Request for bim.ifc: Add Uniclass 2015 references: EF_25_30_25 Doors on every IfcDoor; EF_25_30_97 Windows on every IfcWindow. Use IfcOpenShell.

First a look at what the model holds.

```python
import ifcopenshell

model = ifcopenshell.open("bim.ifc")
print(model.schema)
print("classifications:", [c.Name for c in model.by_type("IfcClassification")])
for ifc_class in ("IfcDoor", "IfcRoof", "IfcStair", "IfcWall", "IfcWindow"):
    print(ifc_class, len(model.by_type(ifc_class)))
```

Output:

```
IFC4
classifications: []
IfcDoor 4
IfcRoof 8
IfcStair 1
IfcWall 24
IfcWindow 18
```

```python
import ifcopenshell
import ifcopenshell.api.classification

model = ifcopenshell.open("bim.ifc")

system = ifcopenshell.api.classification.add_classification(model, classification="Uniclass 2015")

codes = {
    "IfcDoor": ("EF_25_30_25", "Doors"),
    "IfcWindow": ("EF_25_30_97", "Windows"),
}
for ifc_class, (code, name) in codes.items():
    products = model.by_type(ifc_class)
    ifcopenshell.api.classification.add_reference(
        model, products=products, classification=system, identification=code, name=name
    )
    print(code, len(products))

model.write("bim_rev.ifc")
```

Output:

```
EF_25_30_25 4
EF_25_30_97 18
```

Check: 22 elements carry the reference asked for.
